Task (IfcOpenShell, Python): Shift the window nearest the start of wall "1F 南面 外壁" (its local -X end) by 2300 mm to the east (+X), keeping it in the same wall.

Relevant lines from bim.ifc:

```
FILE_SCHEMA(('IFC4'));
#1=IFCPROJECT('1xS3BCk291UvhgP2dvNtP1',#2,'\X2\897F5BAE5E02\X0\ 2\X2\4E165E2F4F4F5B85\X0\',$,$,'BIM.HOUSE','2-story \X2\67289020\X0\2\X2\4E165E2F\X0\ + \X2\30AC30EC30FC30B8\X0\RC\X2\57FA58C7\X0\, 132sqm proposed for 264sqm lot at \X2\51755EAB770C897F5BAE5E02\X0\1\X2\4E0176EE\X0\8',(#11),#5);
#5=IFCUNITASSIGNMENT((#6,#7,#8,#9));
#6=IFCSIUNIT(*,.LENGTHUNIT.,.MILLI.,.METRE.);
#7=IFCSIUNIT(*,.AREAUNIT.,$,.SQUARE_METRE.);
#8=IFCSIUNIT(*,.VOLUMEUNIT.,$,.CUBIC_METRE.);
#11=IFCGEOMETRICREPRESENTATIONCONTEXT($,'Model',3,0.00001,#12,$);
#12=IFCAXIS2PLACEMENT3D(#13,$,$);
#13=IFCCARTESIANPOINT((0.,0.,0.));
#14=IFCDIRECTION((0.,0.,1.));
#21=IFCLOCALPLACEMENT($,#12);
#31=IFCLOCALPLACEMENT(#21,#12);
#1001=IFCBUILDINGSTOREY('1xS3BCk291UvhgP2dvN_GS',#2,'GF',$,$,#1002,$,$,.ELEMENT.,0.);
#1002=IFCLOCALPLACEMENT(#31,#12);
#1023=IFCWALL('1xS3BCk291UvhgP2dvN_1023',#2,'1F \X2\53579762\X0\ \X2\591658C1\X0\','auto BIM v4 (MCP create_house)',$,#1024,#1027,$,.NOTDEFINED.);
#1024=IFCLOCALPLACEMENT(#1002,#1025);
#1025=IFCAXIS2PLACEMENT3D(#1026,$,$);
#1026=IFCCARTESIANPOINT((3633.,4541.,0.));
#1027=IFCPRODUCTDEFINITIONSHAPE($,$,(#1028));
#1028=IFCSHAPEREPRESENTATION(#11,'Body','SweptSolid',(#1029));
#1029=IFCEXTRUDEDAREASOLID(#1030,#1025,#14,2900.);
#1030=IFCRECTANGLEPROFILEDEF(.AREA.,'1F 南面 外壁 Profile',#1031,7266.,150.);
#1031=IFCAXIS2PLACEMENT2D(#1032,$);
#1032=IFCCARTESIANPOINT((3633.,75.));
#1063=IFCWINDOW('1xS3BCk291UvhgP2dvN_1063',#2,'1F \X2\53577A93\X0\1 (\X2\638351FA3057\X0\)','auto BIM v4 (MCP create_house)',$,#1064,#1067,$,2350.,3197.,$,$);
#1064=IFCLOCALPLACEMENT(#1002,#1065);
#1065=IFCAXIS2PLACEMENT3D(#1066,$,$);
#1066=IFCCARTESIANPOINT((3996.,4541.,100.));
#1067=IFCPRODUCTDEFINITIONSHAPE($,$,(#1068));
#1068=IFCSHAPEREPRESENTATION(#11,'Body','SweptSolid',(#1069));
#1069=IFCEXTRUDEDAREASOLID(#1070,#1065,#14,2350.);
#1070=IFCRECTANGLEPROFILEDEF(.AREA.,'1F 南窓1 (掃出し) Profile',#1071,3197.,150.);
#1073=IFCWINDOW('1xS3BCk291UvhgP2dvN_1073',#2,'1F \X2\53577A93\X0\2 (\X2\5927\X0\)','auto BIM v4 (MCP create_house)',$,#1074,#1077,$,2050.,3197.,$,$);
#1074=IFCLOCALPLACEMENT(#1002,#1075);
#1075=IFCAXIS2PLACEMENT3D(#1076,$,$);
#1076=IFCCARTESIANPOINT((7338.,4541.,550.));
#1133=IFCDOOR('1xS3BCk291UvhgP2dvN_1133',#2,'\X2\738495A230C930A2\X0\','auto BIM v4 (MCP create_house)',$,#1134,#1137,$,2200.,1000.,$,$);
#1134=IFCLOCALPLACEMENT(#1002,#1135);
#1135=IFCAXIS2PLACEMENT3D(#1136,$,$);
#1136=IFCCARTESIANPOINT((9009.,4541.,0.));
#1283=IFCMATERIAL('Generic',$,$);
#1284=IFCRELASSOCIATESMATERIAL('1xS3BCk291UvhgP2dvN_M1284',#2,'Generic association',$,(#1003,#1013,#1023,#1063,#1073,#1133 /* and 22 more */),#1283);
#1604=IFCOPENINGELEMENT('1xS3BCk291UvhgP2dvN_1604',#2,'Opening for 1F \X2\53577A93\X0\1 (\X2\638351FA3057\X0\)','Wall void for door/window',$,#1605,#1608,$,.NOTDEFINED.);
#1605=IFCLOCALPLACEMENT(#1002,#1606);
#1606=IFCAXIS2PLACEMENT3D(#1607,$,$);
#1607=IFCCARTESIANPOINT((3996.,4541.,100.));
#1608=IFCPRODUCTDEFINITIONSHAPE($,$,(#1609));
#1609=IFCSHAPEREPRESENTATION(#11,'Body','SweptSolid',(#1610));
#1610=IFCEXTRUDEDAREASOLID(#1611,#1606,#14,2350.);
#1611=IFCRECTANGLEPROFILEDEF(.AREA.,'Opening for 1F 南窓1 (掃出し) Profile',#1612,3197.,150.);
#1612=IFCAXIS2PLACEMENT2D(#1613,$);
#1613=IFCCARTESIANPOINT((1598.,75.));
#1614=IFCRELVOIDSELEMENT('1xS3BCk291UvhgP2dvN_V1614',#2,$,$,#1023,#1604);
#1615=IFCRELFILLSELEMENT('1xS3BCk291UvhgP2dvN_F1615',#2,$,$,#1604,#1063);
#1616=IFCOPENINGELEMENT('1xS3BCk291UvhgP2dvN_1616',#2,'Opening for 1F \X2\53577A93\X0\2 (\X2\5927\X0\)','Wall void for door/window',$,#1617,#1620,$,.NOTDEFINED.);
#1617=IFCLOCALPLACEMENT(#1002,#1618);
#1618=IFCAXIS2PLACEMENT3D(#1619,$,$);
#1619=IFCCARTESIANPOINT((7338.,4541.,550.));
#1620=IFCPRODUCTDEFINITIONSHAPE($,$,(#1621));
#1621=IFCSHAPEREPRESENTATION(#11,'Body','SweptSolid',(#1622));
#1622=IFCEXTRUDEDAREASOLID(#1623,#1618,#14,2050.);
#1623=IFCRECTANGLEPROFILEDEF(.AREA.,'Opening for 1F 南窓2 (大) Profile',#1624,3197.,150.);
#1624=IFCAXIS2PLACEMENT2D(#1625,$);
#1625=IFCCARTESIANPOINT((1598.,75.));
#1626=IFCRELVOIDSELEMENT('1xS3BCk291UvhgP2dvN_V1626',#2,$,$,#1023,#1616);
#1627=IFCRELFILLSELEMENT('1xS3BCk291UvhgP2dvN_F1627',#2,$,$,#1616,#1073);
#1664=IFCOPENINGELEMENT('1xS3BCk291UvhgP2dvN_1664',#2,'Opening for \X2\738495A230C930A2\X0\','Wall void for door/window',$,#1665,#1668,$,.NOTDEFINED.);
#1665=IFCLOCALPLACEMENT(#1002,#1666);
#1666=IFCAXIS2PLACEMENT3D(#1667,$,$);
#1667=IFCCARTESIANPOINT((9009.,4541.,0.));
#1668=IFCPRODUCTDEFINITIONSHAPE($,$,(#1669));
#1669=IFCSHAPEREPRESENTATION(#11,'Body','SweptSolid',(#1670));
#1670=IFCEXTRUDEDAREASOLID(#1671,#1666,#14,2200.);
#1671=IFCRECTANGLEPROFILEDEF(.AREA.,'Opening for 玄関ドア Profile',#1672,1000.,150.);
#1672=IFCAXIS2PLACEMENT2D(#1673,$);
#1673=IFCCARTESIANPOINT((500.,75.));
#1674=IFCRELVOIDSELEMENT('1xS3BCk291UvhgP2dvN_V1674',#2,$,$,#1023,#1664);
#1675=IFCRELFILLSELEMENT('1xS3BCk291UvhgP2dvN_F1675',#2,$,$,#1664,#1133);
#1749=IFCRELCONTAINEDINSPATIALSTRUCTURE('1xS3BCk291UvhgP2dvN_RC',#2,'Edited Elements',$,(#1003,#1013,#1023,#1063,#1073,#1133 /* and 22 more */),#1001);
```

```python
import ifcopenshell
import ifcopenshell.api.geometry
import ifcopenshell.util.placement
import ifcopenshell.util.unit

model = ifcopenshell.open("bim.ifc")
unit_scale = ifcopenshell.util.unit.calculate_unit_scale(model)

window = model.by_guid("1xS3BCk291UvhgP2dvN_1063")
opening = window.FillsVoids[0].RelatingOpeningElement
wall = opening.VoidsElements[0].RelatingBuildingElement

wall_matrix = ifcopenshell.util.placement.get_local_placement(wall.ObjectPlacement)
shift = wall_matrix[:3, 0] * 2.3 / unit_scale
before = ifcopenshell.util.placement.get_local_placement(window.ObjectPlacement)[:3, 3].copy()

# The window is not placed relative to its opening, so move both.
for product in (opening, window):
    matrix = ifcopenshell.util.placement.get_local_placement(product.ObjectPlacement)
    matrix[:3, 3] += shift
    ifcopenshell.api.geometry.edit_object_placement(model, product=product, matrix=matrix, is_si=False)

after = ifcopenshell.util.placement.get_local_placement(window.ObjectPlacement)[:3, 3]
print("window moved by", (after - before).round(3) + 0.0)

model.write("bim_updated.ifc")
```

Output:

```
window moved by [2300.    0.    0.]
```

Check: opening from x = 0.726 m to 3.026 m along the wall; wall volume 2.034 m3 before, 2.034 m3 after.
